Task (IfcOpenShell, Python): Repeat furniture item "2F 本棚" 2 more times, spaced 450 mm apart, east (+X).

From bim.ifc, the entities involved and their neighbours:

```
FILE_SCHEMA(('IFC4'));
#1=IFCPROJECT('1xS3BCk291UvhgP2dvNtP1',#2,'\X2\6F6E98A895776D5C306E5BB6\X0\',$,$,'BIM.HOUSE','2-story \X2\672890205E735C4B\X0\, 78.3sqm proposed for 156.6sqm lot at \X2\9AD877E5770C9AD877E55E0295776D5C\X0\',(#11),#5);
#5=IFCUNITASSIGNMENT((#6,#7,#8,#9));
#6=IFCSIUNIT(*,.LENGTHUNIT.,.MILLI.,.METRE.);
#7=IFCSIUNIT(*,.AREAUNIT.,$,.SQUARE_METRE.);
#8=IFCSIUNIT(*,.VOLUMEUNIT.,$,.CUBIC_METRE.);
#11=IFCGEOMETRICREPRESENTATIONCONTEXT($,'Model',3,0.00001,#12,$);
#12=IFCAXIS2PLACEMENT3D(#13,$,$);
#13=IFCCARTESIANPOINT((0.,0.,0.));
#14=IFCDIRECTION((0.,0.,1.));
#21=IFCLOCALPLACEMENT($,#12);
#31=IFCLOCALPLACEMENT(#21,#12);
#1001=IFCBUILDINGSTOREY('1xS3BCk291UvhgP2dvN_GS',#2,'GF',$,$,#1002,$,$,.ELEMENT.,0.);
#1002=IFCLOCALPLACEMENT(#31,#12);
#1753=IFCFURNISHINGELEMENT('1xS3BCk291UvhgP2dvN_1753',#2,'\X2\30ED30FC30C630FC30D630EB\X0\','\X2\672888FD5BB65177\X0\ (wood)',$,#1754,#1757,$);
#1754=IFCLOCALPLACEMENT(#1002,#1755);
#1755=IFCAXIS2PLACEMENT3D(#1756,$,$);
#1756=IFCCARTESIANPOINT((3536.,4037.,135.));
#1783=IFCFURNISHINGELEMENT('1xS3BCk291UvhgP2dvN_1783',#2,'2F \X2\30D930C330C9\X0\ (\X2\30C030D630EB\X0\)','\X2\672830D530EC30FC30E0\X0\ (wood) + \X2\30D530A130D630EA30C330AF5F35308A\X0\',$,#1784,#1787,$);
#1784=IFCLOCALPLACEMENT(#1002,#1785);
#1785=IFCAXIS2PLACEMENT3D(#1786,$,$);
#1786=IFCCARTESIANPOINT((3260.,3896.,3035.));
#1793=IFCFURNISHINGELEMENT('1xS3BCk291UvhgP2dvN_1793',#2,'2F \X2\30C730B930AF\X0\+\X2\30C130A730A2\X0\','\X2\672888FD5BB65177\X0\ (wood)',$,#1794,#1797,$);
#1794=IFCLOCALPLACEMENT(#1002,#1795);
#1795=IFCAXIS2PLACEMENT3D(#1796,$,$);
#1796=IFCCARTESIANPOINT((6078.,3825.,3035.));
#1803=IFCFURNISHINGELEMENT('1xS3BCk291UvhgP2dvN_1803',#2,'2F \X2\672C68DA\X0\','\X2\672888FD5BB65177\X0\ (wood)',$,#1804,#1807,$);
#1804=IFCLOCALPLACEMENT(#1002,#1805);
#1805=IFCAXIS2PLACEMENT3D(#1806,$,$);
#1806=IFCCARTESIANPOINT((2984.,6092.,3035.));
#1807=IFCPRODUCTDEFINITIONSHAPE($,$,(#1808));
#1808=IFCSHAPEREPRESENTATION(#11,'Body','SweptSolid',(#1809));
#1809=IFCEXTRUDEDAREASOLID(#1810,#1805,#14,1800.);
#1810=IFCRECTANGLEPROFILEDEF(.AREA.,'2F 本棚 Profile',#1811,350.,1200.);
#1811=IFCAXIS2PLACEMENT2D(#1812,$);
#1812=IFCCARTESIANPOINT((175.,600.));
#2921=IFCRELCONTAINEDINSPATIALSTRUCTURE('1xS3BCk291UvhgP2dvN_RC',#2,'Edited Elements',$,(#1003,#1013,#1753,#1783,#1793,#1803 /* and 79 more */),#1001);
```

```python
import numpy as np
import ifcopenshell
import ifcopenshell.api.geometry
import ifcopenshell.api.root
import ifcopenshell.util.element
import ifcopenshell.util.placement
import ifcopenshell.util.unit

model = ifcopenshell.open("bim.ifc")
unit_scale = ifcopenshell.util.unit.calculate_unit_scale(model)


def reuse_history(source, copy):
    """copy_class also copies each property set's owner history, people and application; keep the originals."""
    for rel in copy.IsDefinedBy:
        if rel.is_a("IfcRelDefinesByProperties") and (history := rel.RelatingPropertyDefinition.OwnerHistory):
            rel.RelatingPropertyDefinition.OwnerHistory = source.OwnerHistory
            ifcopenshell.util.element.remove_deep2(model, history)


source = model.by_guid("1xS3BCk291UvhgP2dvN_1803")
base = ifcopenshell.util.placement.get_local_placement(source.ObjectPlacement)
step = np.array([1.0, 0.0, 0.0]) * 0.45 / unit_scale

for i in range(1, 3):
    copy = ifcopenshell.api.root.copy_class(model, product=source)
    copy.Representation = ifcopenshell.util.element.copy_deep(
        model, source.Representation, exclude=["IfcGeometricRepresentationContext", "IfcRepresentationMap"]
    )
    reuse_history(source, copy)
    matrix = base.copy()
    matrix[:3, 3] += i * step
    print("added at", matrix[:3, 3].round(3) + 0.0)
    ifcopenshell.api.geometry.edit_object_placement(model, product=copy, matrix=matrix, is_si=False)

model.write("bim_rev.ifc")
```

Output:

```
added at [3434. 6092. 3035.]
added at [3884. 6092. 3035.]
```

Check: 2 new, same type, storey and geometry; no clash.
